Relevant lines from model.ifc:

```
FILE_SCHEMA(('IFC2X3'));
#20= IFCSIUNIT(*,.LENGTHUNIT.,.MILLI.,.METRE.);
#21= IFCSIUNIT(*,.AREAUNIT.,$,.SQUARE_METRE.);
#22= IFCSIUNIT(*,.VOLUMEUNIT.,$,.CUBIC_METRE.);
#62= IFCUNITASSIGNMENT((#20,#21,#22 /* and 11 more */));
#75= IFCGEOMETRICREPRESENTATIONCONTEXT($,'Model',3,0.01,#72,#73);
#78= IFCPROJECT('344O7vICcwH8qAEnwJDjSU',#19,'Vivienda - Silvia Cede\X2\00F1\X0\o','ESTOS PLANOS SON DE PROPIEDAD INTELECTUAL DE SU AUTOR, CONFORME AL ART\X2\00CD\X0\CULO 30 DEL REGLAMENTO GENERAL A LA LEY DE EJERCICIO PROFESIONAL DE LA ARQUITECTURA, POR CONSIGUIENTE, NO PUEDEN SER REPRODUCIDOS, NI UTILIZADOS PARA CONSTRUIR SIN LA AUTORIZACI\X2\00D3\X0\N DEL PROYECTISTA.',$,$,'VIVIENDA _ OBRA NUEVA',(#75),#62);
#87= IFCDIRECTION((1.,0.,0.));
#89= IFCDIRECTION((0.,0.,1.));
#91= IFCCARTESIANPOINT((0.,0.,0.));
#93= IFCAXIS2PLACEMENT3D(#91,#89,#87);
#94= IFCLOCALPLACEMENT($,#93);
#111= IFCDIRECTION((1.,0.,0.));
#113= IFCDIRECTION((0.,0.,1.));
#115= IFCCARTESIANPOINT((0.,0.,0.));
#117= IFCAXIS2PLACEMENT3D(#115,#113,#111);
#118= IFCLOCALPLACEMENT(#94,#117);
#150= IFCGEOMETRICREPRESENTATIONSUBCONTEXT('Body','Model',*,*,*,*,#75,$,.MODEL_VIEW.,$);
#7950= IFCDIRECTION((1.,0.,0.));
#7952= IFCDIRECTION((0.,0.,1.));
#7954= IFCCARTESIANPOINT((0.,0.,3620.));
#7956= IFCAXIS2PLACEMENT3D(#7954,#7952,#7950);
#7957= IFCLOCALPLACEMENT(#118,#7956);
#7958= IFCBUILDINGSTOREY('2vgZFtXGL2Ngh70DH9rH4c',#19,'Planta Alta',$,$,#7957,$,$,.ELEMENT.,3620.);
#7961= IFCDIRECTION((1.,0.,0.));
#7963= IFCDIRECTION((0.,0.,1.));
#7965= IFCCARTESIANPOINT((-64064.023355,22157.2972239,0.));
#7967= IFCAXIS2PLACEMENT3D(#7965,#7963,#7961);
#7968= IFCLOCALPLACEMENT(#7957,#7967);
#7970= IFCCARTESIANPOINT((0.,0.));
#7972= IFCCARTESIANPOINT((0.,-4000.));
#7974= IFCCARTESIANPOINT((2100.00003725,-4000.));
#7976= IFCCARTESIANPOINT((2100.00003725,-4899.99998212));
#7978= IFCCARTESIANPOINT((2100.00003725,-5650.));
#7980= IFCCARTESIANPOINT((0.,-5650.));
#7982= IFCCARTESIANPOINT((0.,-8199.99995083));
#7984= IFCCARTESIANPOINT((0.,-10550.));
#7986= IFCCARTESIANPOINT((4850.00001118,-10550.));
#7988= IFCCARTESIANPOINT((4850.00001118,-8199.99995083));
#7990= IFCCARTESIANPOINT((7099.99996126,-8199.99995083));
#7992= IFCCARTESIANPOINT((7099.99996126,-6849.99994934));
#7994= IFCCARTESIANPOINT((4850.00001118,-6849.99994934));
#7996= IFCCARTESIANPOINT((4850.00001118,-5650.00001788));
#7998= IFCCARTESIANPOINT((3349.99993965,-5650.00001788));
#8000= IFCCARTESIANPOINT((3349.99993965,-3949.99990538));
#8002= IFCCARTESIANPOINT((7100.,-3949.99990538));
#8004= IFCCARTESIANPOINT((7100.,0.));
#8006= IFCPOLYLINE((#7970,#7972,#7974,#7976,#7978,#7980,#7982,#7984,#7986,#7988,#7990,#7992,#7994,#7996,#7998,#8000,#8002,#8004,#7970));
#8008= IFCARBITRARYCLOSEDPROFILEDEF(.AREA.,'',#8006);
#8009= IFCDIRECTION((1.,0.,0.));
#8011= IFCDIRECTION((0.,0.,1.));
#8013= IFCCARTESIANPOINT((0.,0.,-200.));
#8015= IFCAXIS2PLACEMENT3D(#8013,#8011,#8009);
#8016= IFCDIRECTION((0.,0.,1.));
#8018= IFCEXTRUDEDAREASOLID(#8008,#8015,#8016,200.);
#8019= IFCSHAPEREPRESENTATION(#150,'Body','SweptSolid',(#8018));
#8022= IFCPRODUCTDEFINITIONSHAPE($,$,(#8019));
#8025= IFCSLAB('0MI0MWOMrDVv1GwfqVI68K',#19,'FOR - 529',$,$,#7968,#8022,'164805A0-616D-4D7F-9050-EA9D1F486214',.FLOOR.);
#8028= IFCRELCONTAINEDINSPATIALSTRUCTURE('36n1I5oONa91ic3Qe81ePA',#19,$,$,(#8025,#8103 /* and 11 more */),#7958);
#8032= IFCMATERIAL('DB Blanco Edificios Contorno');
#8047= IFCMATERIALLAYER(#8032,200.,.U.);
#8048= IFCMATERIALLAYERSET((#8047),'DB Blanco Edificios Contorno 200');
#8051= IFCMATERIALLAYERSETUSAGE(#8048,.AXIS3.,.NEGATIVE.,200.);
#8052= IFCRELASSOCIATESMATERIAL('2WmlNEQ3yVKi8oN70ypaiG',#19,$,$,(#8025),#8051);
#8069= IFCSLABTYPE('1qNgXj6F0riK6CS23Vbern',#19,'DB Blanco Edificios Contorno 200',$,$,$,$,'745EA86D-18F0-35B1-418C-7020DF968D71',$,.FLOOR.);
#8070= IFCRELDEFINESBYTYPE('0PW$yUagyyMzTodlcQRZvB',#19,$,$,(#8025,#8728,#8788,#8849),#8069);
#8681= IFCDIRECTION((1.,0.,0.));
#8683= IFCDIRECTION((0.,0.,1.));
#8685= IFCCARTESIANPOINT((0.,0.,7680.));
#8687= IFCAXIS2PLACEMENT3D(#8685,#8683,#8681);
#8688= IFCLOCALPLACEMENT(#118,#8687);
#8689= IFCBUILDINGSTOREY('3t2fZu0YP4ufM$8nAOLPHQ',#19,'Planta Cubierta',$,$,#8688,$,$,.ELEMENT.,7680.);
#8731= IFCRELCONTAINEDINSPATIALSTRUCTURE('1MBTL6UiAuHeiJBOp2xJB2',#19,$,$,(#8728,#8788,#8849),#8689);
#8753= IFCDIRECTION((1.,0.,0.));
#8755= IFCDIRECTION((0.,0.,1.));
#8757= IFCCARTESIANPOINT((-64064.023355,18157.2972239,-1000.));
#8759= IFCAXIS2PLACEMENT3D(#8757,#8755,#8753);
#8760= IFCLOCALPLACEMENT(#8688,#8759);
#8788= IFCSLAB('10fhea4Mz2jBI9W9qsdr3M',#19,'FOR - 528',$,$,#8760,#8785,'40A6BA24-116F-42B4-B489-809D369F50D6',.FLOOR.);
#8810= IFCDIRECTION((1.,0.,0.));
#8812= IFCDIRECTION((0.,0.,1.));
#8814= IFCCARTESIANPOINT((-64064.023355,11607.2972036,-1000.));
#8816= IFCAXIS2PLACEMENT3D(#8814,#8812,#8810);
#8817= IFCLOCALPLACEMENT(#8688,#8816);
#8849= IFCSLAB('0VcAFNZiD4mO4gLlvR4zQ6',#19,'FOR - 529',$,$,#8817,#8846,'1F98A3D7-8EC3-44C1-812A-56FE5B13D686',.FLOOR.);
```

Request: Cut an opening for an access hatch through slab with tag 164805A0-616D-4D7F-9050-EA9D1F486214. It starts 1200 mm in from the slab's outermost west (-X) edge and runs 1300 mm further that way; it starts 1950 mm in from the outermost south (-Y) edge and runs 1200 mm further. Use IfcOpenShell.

```python
import numpy as np
import ifcopenshell
import ifcopenshell.api.feature
import ifcopenshell.api.geometry
import ifcopenshell.api.root
import ifcopenshell.geom
import ifcopenshell.util.placement
import ifcopenshell.util.representation
import ifcopenshell.util.shape
import ifcopenshell.util.unit

model = ifcopenshell.open("model.ifc")
unit_scale = ifcopenshell.util.unit.calculate_unit_scale(model)
settings = ifcopenshell.geom.settings()


def volume(element):
    """Net volume in cubic metres, openings subtracted."""
    shape = ifcopenshell.geom.create_shape(settings, element)
    return ifcopenshell.util.shape.get_volume(shape.geometry)


slab = model.by_id(8025)
before = volume(slab)

# Extent in the slab's own axes, in metres. The edges named are its -X and -Y sides.
slab_shape = ifcopenshell.geom.create_shape(settings, slab)
vertices = ifcopenshell.util.shape.get_vertices(slab_shape.geometry)
x_min, y_min, bottom = vertices.min(axis=0)
top = vertices[:, 2].max()

opening = ifcopenshell.api.root.create_entity(model, ifc_class="IfcOpeningElement", name="Access hatch opening")
context = ifcopenshell.util.representation.get_context(model, "Model", "Body", "MODEL_VIEW")
width, depth = 1.3, 1.2
outline = [(0.0, 0.0), (width, 0.0), (width, depth), (0.0, depth), (0.0, 0.0)]
# Overshoot both faces by 50 mm so the cut is clean.
shape = ifcopenshell.api.geometry.add_slab_representation(
    model, context=context, depth=top - bottom + 0.1, polyline=outline
)
ifcopenshell.api.geometry.assign_representation(model, product=opening, representation=shape)

matrix = ifcopenshell.util.placement.get_local_placement(slab.ObjectPlacement)
matrix[:, 3] = matrix @ np.append(np.array([x_min + 1.2, y_min + 1.95, bottom - 0.05]) / unit_scale, 1.0)
ifcopenshell.api.geometry.edit_object_placement(model, product=opening, matrix=matrix, is_si=False)
ifcopenshell.api.feature.add_feature(model, feature=opening, element=slab)

after = volume(slab)

print(f"slab volume {before:.3f} -> {after:.3f} m3")

model.write("model-out.ifc")
```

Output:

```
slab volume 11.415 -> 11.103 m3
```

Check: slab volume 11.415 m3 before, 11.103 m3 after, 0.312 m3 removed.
